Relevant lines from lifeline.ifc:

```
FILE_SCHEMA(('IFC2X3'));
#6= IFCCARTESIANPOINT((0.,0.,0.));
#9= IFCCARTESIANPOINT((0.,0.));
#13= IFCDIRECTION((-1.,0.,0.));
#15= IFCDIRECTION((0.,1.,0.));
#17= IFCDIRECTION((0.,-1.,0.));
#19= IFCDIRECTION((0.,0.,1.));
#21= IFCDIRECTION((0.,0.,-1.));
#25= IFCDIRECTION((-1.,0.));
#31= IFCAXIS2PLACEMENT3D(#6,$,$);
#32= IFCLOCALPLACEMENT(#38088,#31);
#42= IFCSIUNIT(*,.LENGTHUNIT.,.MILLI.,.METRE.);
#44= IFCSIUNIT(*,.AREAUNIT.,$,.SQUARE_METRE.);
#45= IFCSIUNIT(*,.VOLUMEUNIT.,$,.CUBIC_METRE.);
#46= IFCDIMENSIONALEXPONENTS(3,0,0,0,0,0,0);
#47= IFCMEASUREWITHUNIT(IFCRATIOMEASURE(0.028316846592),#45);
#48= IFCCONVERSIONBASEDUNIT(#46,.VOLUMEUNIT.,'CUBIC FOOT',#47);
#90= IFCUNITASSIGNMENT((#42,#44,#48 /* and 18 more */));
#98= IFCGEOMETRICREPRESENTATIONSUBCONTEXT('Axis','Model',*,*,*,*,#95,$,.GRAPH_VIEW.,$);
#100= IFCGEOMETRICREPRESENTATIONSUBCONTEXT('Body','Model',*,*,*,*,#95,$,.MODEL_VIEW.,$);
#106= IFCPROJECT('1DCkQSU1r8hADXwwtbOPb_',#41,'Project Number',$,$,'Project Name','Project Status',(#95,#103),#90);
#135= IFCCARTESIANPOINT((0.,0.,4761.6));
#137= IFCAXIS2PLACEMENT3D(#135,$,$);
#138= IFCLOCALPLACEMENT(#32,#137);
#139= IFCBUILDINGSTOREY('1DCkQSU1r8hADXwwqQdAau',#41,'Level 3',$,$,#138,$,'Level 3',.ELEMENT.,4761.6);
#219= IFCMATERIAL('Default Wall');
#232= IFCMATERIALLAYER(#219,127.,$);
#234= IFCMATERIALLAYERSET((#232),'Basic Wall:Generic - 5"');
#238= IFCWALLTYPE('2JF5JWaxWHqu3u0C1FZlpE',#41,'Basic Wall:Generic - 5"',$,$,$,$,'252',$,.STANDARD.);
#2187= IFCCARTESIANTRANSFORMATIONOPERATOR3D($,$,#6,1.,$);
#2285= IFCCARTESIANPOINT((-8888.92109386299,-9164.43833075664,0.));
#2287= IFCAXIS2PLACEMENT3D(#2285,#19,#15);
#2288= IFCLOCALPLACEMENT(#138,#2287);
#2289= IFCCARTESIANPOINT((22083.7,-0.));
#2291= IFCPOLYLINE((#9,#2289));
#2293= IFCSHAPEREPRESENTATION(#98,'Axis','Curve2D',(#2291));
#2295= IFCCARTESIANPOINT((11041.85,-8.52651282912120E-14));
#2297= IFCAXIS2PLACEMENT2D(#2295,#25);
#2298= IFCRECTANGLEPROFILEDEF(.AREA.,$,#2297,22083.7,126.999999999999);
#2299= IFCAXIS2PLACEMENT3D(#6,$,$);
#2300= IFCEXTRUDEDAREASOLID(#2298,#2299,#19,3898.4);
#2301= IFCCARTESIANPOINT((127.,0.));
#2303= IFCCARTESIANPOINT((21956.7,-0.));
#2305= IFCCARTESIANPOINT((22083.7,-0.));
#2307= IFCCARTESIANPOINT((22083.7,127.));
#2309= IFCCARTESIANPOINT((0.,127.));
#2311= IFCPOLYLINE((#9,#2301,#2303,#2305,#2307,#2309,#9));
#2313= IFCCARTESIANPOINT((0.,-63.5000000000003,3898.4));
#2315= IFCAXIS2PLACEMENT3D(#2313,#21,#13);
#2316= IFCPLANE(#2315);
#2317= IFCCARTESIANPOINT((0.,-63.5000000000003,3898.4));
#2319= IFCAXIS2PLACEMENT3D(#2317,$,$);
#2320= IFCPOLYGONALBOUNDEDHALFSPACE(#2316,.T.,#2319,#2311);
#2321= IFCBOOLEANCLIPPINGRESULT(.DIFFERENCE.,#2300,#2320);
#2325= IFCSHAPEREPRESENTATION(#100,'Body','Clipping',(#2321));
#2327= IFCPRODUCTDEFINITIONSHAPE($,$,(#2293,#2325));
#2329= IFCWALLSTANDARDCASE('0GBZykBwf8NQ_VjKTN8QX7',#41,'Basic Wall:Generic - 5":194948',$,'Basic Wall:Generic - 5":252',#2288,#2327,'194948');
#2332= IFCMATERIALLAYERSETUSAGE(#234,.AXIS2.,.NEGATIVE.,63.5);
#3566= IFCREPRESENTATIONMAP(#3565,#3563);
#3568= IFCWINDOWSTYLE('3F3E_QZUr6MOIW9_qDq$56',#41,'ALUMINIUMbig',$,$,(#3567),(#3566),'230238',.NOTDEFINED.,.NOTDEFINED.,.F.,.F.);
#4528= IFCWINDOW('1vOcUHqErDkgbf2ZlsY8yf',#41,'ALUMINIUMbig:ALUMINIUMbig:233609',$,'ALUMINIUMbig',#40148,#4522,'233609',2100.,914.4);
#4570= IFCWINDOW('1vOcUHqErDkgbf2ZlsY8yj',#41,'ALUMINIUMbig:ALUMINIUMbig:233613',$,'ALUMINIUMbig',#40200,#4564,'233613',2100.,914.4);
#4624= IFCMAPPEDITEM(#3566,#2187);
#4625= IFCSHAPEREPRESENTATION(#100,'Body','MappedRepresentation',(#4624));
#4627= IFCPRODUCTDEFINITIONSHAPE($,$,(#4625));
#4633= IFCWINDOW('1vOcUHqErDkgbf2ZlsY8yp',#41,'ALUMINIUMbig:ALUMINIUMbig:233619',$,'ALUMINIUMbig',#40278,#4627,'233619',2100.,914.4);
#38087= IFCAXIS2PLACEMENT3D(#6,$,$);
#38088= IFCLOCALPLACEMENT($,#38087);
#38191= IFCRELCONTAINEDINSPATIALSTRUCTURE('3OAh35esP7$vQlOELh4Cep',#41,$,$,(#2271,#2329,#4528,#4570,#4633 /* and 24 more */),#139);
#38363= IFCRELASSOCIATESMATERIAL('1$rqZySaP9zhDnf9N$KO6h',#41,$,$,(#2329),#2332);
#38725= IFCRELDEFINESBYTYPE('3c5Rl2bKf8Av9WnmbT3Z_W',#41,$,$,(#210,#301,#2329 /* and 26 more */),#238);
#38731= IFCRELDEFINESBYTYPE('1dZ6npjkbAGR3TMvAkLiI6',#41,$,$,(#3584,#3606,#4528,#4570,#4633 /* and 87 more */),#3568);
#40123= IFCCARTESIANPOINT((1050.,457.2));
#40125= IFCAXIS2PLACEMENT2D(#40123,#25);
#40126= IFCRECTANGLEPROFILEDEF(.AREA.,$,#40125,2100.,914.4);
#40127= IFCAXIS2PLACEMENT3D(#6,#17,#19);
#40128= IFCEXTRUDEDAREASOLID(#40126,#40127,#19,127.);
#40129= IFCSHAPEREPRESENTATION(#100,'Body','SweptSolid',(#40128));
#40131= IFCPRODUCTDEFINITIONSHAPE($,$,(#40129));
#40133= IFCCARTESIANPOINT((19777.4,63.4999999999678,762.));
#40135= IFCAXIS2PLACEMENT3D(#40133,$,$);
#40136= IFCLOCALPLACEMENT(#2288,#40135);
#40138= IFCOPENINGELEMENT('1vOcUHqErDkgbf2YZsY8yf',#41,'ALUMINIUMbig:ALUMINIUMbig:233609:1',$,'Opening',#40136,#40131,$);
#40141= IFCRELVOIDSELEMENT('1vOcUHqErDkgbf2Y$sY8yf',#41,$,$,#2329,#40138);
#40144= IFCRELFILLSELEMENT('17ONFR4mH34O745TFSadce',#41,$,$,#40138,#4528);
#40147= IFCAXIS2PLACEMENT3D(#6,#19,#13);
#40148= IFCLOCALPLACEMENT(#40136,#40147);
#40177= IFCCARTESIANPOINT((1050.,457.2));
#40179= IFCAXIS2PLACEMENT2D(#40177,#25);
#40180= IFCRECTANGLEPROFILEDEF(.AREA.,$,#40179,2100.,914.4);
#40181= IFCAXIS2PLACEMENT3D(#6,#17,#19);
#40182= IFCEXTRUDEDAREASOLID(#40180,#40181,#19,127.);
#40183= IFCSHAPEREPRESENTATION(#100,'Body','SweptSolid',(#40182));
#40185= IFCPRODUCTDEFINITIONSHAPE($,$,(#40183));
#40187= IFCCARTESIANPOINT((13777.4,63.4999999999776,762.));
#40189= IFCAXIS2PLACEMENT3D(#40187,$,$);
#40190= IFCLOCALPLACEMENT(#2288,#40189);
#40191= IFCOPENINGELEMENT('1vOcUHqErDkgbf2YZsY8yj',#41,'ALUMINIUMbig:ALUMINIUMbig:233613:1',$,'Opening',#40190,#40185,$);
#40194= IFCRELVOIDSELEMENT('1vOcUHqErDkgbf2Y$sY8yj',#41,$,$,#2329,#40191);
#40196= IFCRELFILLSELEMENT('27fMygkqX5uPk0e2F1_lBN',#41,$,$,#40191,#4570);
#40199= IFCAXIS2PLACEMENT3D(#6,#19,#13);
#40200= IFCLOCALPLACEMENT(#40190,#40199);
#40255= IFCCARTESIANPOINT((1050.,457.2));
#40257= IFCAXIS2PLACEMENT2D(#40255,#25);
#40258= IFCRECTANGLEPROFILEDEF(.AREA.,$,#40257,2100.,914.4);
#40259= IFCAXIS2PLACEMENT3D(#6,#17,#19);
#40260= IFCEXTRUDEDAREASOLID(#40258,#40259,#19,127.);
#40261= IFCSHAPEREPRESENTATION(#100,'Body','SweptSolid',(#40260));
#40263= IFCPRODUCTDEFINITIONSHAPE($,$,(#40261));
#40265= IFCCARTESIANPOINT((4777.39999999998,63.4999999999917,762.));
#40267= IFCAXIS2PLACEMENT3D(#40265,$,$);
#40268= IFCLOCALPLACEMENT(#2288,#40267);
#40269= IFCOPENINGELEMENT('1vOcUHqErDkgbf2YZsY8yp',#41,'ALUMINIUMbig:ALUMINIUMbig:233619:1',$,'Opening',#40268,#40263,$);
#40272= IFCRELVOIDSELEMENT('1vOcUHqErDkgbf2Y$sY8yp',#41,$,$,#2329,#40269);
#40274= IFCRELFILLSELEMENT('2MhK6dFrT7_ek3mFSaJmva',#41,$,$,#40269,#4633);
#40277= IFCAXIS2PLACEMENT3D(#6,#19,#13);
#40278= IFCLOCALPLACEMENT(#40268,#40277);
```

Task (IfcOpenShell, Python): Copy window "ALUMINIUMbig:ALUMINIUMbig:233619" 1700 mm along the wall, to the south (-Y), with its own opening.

```python
import ifcopenshell
import ifcopenshell.api.feature
import ifcopenshell.api.geometry
import ifcopenshell.api.root
import ifcopenshell.geom
import ifcopenshell.util.element
import ifcopenshell.util.placement
import ifcopenshell.util.shape
import ifcopenshell.util.unit

model = ifcopenshell.open("lifeline.ifc")
unit_scale = ifcopenshell.util.unit.calculate_unit_scale(model)
settings = ifcopenshell.geom.settings()


def volume(element):
    """Net volume in cubic metres, openings subtracted."""
    shape = ifcopenshell.geom.create_shape(settings, element)
    return ifcopenshell.util.shape.get_volume(shape.geometry)


def reuse_history(source, copy):
    """copy_class also copies each property set's owner history, people and application; keep the originals."""
    for rel in copy.IsDefinedBy:
        if rel.is_a("IfcRelDefinesByProperties") and (history := rel.RelatingPropertyDefinition.OwnerHistory):
            rel.RelatingPropertyDefinition.OwnerHistory = source.OwnerHistory
            ifcopenshell.util.element.remove_deep2(model, history)


window = model.by_guid("1vOcUHqErDkgbf2ZlsY8yp")
opening = window.FillsVoids[0].RelatingOpeningElement
wall = opening.VoidsElements[0].RelatingBuildingElement
before = volume(wall)
shift = ifcopenshell.util.placement.get_local_placement(wall.ObjectPlacement)[:3, 0] * -1.7 / unit_scale

# copy_class copies the void relationship, type, container and properties, but no geometry.
new_opening = ifcopenshell.api.root.copy_class(model, product=opening)
new_opening.Representation = ifcopenshell.util.element.copy_deep(
    model, opening.Representation, exclude=["IfcGeometricRepresentationContext", "IfcRepresentationMap"]
)
new_opening.Name = "ALUMINIUMbig:ALUMINIUMbig"
new_window = ifcopenshell.api.root.copy_class(model, product=window)
new_window.Representation = ifcopenshell.util.element.copy_deep(
    model, window.Representation, exclude=["IfcGeometricRepresentationContext", "IfcRepresentationMap"]
)
new_window.Name = "ALUMINIUMbig:ALUMINIUMbig"
new_window.Tag = None
reuse_history(window, new_window)
fills = ifcopenshell.api.feature.add_filling(model, opening=new_opening, element=new_window)
fills.OwnerHistory = new_window.OwnerHistory  # required in IFC2X3

for old, new in ((opening, new_opening), (window, new_window)):
    matrix = ifcopenshell.util.placement.get_local_placement(old.ObjectPlacement)
    matrix[:3, 3] += shift
    ifcopenshell.api.geometry.edit_object_placement(model, product=new, matrix=matrix, is_si=False)

after = volume(wall)

print(f"wall volume {before:.3f} -> {after:.3f} m3")

model.write("lifeline_rev.ifc")
```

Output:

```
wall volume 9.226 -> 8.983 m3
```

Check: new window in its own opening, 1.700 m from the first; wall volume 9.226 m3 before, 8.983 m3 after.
